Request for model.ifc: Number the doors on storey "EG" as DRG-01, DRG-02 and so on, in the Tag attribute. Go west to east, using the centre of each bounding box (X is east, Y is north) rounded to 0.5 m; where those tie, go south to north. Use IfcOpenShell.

First a look at what the model holds.

```python
import ifcopenshell
import ifcopenshell.util.element
import ifcopenshell.util.placement

model = ifcopenshell.open("model.ifc")
print(model.schema)
storey = next(s for s in model.by_type("IfcBuildingStorey") if s.Name == "EG")
doors = [e for e in ifcopenshell.util.element.get_decomposition(storey) if e.is_a("IfcDoor")]
for e in sorted(doors, key=lambda e: e.id()):
    origin = ifcopenshell.util.placement.get_local_placement(e.ObjectPlacement)[:3, 3]
    print(e.id(), e.Tag, e.Name, origin.round(2) + 0.0, sep=" | ")
```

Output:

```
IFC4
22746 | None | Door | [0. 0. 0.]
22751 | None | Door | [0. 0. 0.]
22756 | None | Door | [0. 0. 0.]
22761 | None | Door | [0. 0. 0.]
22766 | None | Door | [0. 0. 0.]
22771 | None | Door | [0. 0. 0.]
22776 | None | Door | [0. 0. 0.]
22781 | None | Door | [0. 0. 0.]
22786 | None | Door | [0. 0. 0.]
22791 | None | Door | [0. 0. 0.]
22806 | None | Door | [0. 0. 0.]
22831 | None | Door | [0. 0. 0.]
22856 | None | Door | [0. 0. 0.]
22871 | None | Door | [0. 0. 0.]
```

```python
import ifcopenshell
import ifcopenshell.geom
import ifcopenshell.util.element
import ifcopenshell.util.shape

model = ifcopenshell.open("model.ifc")
settings = ifcopenshell.geom.settings()
settings.set("use-world-coords", True)


def centre(element):
    shape = ifcopenshell.geom.create_shape(settings, element)
    return ifcopenshell.util.shape.get_bbox_centroid(shape.geometry)


storey = next(s for s in model.by_type("IfcBuildingStorey") if s.Name == "EG")
doors = [e for e in ifcopenshell.util.element.get_decomposition(storey) if e.is_a("IfcDoor")]

# Insertion points can sit at a corner or the storey origin, so sort by the geometry (in metres).
centres = {e: centre(e) for e in doors}
doors.sort(key=lambda e: (round(centres[e][0] / 0.5), centres[e][1]))

for i, e in enumerate(doors, start=1):
    number = f"DRG-{i:02d}"
    e.Tag = number
    print(e.id(), number)

model.write("model_updated.ifc")
```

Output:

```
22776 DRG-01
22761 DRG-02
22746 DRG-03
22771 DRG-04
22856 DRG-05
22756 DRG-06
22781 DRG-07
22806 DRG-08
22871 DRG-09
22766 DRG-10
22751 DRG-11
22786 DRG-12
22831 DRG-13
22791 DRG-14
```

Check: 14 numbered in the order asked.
